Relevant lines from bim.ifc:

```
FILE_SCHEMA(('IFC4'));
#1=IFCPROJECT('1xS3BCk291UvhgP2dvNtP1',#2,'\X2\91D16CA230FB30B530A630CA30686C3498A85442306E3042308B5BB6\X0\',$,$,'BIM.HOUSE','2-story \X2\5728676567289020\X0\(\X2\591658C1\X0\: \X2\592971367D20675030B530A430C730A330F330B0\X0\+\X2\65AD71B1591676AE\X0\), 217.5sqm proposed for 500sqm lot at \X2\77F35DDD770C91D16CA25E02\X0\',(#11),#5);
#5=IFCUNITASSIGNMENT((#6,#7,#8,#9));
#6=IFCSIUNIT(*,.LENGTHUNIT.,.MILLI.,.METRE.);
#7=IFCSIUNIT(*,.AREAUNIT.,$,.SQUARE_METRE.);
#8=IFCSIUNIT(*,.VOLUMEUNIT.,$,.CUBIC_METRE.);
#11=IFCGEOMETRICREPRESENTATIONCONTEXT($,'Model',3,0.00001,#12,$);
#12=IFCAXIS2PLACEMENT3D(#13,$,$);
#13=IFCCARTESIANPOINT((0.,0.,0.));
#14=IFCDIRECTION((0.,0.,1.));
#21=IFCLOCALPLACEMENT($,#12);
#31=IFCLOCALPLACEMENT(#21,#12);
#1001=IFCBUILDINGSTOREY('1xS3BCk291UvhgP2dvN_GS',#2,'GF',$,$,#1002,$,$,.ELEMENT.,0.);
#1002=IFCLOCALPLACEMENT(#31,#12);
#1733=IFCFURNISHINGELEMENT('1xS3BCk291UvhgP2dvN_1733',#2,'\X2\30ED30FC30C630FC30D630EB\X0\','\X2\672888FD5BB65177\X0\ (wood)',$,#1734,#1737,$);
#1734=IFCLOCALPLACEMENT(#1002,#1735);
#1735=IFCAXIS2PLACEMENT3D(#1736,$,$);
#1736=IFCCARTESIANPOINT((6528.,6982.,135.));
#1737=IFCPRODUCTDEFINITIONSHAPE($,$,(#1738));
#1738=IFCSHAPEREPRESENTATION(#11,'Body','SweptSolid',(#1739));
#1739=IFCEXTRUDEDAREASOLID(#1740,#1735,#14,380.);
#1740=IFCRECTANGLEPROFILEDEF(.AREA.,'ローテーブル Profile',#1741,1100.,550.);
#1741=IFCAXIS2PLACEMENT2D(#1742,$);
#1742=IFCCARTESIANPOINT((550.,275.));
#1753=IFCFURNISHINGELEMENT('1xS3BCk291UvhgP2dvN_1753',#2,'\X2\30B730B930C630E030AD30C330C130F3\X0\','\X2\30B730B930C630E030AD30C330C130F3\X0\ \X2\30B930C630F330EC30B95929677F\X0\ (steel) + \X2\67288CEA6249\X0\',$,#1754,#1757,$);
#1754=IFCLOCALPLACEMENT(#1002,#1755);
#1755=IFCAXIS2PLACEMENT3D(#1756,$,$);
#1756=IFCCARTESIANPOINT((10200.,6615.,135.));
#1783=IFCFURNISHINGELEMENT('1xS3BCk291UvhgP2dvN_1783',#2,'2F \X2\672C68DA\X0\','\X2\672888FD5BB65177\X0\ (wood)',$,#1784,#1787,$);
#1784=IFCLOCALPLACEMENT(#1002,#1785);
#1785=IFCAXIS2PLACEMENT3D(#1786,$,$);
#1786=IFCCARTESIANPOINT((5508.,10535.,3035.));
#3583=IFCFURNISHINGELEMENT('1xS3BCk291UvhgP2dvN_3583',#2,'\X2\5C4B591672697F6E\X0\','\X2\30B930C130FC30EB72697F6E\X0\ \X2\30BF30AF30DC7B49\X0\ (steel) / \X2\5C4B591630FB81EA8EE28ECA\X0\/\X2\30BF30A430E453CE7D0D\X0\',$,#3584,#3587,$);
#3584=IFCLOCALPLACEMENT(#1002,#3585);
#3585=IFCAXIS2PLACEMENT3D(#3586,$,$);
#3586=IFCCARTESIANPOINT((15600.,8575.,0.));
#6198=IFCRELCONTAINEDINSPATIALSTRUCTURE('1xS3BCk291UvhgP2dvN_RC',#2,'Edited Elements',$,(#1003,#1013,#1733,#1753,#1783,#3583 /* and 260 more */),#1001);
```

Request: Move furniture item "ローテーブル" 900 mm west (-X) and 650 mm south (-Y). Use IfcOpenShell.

```python
import ifcopenshell
import ifcopenshell.api.geometry
import ifcopenshell.util.placement
import ifcopenshell.util.unit

model = ifcopenshell.open("bim.ifc")
unit_scale = ifcopenshell.util.unit.calculate_unit_scale(model)

item = model.by_guid("1xS3BCk291UvhgP2dvN_1733")
matrix = ifcopenshell.util.placement.get_local_placement(item.ObjectPlacement)
matrix[0, 3] -= 0.9 / unit_scale
matrix[1, 3] -= 0.65 / unit_scale
ifcopenshell.api.geometry.edit_object_placement(model, product=item, matrix=matrix, is_si=False)

print(ifcopenshell.util.placement.get_local_placement(item.ObjectPlacement).round(3) + 0.0)

model.write("bim_rev.ifc")
```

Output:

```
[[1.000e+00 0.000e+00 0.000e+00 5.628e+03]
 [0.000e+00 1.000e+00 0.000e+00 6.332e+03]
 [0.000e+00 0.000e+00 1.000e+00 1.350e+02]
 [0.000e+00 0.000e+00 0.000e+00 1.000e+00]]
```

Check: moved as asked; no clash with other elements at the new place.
